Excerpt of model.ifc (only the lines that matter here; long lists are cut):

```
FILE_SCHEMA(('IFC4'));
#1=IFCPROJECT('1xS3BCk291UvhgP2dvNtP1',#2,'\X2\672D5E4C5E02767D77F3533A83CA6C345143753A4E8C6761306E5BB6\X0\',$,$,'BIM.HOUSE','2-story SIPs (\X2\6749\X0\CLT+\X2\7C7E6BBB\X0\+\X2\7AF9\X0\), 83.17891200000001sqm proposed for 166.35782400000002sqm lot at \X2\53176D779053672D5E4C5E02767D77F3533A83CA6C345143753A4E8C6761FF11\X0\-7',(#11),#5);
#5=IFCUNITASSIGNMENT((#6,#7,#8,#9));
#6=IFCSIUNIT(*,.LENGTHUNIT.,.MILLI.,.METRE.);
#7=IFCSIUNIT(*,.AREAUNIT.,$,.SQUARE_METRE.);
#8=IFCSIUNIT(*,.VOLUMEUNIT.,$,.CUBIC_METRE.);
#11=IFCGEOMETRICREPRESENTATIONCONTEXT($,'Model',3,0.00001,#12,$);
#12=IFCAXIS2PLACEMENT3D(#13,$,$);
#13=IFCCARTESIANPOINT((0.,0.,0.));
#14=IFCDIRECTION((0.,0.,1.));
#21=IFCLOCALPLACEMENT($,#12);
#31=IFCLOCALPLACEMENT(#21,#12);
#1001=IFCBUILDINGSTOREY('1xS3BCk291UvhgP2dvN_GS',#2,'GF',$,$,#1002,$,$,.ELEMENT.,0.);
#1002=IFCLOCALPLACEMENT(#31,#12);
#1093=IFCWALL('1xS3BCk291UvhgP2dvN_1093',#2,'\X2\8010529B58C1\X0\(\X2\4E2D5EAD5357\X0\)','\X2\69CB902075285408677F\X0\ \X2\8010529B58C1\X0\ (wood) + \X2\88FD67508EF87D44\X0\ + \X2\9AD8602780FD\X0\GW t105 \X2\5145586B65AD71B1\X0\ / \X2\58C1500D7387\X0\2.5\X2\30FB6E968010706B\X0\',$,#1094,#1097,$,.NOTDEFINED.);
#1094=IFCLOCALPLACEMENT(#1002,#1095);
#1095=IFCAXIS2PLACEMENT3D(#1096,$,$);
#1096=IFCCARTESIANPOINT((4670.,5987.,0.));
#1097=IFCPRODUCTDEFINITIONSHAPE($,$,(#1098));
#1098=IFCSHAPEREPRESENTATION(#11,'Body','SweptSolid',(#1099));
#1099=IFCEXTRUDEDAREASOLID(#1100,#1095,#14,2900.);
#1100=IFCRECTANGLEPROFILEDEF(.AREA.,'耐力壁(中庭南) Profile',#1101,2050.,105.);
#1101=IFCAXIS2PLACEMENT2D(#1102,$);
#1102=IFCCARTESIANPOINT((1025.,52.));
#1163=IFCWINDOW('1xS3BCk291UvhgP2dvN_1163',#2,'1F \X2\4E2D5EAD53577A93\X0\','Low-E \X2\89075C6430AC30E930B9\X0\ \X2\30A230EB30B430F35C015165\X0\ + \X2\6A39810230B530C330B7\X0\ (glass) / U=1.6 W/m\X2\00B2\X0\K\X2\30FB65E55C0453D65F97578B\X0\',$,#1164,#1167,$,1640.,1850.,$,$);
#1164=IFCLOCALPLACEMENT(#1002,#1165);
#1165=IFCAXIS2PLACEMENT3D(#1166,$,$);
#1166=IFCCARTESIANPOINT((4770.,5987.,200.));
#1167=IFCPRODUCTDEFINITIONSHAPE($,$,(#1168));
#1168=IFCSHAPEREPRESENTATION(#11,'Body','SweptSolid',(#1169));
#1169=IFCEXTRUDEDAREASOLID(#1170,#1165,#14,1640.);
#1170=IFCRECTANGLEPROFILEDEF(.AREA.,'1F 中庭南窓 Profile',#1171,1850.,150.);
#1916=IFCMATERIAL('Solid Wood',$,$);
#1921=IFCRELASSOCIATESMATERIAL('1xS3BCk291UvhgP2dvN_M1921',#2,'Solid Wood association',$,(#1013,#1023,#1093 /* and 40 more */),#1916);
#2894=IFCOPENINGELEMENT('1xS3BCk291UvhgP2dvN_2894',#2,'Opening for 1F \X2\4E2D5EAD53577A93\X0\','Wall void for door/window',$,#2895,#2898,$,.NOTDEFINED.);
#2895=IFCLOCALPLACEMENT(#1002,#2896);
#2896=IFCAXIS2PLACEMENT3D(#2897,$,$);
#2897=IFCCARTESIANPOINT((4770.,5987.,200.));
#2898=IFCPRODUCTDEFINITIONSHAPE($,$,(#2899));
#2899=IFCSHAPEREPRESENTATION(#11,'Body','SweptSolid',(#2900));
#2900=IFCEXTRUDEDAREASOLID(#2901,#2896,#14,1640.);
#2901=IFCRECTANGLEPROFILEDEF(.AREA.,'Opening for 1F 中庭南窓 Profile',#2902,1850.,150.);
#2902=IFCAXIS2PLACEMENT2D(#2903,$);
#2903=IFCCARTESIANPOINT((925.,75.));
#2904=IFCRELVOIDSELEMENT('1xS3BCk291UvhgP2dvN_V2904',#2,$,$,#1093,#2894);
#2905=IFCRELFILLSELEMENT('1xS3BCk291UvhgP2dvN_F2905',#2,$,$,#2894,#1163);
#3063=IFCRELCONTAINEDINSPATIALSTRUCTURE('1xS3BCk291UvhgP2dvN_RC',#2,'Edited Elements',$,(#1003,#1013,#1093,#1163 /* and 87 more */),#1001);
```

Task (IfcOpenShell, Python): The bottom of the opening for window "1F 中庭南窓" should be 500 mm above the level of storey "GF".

```python
import numpy as np
import ifcopenshell
import ifcopenshell.api.geometry
import ifcopenshell.geom
import ifcopenshell.util.element
import ifcopenshell.util.placement
import ifcopenshell.util.shape
import ifcopenshell.util.unit

model = ifcopenshell.open("model.ifc")
unit_scale = ifcopenshell.util.unit.calculate_unit_scale(model)

window = model.by_guid("1xS3BCk291UvhgP2dvN_1163")
opening = window.FillsVoids[0].RelatingOpeningElement
storey = ifcopenshell.util.element.get_container(window, ifc_class="IfcBuildingStorey")
level = ifcopenshell.util.placement.get_local_placement(storey.ObjectPlacement)[2, 3]

# The opening's origin need not be at the sill, so measure its lowest point.
shape = ifcopenshell.geom.create_shape(ifcopenshell.geom.settings(), opening)
bottom = ifcopenshell.util.shape.get_shape_bottom_elevation(shape, shape.geometry) / unit_scale
dz = level + 0.5 / unit_scale - bottom

shift = np.array([0.0, 0.0, dz])
# The window is not placed relative to its opening, so move both.
for product in (opening, window):
    matrix = ifcopenshell.util.placement.get_local_placement(product.ObjectPlacement)
    matrix[:3, 3] += shift
    ifcopenshell.api.geometry.edit_object_placement(model, product=product, matrix=matrix, is_si=False)

print(f"moved by {dz * unit_scale:+.3f} m")

model.write("model_v2.ifc")
```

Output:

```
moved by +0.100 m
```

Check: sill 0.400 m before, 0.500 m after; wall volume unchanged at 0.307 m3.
